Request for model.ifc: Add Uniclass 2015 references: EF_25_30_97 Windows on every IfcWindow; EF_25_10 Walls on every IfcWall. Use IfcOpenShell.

First a look at what the model holds.

```python
import ifcopenshell

model = ifcopenshell.open("model.ifc")
print(model.schema)
print("classifications:", [c.Name for c in model.by_type("IfcClassification")])
for ifc_class in ("IfcDoor", "IfcRoof", "IfcStair", "IfcWall", "IfcWindow"):
    print(ifc_class, len(model.by_type(ifc_class)))
```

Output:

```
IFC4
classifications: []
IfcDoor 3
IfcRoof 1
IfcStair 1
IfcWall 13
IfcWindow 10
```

```python
import ifcopenshell
import ifcopenshell.api.classification

model = ifcopenshell.open("model.ifc")

system = ifcopenshell.api.classification.add_classification(model, classification="Uniclass 2015")

codes = {
    "IfcWindow": ("EF_25_30_97", "Windows"),
    "IfcWall": ("EF_25_10", "Walls"),
}
for ifc_class, (code, name) in codes.items():
    products = model.by_type(ifc_class)
    ifcopenshell.api.classification.add_reference(
        model, products=products, classification=system, identification=code, name=name
    )
    print(code, len(products))

model.write("model_rev.ifc")
```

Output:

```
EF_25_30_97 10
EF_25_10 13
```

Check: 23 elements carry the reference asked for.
